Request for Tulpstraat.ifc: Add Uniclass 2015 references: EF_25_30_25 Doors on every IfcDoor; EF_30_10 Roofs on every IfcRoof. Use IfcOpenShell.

First a look at what the model holds.

```python
import ifcopenshell

model = ifcopenshell.open("Tulpstraat.ifc")
print(model.schema)
print("classifications:", [c.Name for c in model.by_type("IfcClassification")])
for ifc_class in ("IfcDoor", "IfcRoof", "IfcStair", "IfcWall", "IfcWindow"):
    print(ifc_class, len(model.by_type(ifc_class)))
```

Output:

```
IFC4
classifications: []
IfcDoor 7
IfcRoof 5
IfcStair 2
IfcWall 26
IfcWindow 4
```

```python
import ifcopenshell
import ifcopenshell.api.classification

model = ifcopenshell.open("Tulpstraat.ifc")

system = ifcopenshell.api.classification.add_classification(model, classification="Uniclass 2015")

codes = {
    "IfcDoor": ("EF_25_30_25", "Doors"),
    "IfcRoof": ("EF_30_10", "Roofs"),
}
for ifc_class, (code, name) in codes.items():
    products = model.by_type(ifc_class)
    ifcopenshell.api.classification.add_reference(
        model, products=products, classification=system, identification=code, name=name
    )
    print(code, len(products))

model.write("Tulpstraat_updated.ifc")
```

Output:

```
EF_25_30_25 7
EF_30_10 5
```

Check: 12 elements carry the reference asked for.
